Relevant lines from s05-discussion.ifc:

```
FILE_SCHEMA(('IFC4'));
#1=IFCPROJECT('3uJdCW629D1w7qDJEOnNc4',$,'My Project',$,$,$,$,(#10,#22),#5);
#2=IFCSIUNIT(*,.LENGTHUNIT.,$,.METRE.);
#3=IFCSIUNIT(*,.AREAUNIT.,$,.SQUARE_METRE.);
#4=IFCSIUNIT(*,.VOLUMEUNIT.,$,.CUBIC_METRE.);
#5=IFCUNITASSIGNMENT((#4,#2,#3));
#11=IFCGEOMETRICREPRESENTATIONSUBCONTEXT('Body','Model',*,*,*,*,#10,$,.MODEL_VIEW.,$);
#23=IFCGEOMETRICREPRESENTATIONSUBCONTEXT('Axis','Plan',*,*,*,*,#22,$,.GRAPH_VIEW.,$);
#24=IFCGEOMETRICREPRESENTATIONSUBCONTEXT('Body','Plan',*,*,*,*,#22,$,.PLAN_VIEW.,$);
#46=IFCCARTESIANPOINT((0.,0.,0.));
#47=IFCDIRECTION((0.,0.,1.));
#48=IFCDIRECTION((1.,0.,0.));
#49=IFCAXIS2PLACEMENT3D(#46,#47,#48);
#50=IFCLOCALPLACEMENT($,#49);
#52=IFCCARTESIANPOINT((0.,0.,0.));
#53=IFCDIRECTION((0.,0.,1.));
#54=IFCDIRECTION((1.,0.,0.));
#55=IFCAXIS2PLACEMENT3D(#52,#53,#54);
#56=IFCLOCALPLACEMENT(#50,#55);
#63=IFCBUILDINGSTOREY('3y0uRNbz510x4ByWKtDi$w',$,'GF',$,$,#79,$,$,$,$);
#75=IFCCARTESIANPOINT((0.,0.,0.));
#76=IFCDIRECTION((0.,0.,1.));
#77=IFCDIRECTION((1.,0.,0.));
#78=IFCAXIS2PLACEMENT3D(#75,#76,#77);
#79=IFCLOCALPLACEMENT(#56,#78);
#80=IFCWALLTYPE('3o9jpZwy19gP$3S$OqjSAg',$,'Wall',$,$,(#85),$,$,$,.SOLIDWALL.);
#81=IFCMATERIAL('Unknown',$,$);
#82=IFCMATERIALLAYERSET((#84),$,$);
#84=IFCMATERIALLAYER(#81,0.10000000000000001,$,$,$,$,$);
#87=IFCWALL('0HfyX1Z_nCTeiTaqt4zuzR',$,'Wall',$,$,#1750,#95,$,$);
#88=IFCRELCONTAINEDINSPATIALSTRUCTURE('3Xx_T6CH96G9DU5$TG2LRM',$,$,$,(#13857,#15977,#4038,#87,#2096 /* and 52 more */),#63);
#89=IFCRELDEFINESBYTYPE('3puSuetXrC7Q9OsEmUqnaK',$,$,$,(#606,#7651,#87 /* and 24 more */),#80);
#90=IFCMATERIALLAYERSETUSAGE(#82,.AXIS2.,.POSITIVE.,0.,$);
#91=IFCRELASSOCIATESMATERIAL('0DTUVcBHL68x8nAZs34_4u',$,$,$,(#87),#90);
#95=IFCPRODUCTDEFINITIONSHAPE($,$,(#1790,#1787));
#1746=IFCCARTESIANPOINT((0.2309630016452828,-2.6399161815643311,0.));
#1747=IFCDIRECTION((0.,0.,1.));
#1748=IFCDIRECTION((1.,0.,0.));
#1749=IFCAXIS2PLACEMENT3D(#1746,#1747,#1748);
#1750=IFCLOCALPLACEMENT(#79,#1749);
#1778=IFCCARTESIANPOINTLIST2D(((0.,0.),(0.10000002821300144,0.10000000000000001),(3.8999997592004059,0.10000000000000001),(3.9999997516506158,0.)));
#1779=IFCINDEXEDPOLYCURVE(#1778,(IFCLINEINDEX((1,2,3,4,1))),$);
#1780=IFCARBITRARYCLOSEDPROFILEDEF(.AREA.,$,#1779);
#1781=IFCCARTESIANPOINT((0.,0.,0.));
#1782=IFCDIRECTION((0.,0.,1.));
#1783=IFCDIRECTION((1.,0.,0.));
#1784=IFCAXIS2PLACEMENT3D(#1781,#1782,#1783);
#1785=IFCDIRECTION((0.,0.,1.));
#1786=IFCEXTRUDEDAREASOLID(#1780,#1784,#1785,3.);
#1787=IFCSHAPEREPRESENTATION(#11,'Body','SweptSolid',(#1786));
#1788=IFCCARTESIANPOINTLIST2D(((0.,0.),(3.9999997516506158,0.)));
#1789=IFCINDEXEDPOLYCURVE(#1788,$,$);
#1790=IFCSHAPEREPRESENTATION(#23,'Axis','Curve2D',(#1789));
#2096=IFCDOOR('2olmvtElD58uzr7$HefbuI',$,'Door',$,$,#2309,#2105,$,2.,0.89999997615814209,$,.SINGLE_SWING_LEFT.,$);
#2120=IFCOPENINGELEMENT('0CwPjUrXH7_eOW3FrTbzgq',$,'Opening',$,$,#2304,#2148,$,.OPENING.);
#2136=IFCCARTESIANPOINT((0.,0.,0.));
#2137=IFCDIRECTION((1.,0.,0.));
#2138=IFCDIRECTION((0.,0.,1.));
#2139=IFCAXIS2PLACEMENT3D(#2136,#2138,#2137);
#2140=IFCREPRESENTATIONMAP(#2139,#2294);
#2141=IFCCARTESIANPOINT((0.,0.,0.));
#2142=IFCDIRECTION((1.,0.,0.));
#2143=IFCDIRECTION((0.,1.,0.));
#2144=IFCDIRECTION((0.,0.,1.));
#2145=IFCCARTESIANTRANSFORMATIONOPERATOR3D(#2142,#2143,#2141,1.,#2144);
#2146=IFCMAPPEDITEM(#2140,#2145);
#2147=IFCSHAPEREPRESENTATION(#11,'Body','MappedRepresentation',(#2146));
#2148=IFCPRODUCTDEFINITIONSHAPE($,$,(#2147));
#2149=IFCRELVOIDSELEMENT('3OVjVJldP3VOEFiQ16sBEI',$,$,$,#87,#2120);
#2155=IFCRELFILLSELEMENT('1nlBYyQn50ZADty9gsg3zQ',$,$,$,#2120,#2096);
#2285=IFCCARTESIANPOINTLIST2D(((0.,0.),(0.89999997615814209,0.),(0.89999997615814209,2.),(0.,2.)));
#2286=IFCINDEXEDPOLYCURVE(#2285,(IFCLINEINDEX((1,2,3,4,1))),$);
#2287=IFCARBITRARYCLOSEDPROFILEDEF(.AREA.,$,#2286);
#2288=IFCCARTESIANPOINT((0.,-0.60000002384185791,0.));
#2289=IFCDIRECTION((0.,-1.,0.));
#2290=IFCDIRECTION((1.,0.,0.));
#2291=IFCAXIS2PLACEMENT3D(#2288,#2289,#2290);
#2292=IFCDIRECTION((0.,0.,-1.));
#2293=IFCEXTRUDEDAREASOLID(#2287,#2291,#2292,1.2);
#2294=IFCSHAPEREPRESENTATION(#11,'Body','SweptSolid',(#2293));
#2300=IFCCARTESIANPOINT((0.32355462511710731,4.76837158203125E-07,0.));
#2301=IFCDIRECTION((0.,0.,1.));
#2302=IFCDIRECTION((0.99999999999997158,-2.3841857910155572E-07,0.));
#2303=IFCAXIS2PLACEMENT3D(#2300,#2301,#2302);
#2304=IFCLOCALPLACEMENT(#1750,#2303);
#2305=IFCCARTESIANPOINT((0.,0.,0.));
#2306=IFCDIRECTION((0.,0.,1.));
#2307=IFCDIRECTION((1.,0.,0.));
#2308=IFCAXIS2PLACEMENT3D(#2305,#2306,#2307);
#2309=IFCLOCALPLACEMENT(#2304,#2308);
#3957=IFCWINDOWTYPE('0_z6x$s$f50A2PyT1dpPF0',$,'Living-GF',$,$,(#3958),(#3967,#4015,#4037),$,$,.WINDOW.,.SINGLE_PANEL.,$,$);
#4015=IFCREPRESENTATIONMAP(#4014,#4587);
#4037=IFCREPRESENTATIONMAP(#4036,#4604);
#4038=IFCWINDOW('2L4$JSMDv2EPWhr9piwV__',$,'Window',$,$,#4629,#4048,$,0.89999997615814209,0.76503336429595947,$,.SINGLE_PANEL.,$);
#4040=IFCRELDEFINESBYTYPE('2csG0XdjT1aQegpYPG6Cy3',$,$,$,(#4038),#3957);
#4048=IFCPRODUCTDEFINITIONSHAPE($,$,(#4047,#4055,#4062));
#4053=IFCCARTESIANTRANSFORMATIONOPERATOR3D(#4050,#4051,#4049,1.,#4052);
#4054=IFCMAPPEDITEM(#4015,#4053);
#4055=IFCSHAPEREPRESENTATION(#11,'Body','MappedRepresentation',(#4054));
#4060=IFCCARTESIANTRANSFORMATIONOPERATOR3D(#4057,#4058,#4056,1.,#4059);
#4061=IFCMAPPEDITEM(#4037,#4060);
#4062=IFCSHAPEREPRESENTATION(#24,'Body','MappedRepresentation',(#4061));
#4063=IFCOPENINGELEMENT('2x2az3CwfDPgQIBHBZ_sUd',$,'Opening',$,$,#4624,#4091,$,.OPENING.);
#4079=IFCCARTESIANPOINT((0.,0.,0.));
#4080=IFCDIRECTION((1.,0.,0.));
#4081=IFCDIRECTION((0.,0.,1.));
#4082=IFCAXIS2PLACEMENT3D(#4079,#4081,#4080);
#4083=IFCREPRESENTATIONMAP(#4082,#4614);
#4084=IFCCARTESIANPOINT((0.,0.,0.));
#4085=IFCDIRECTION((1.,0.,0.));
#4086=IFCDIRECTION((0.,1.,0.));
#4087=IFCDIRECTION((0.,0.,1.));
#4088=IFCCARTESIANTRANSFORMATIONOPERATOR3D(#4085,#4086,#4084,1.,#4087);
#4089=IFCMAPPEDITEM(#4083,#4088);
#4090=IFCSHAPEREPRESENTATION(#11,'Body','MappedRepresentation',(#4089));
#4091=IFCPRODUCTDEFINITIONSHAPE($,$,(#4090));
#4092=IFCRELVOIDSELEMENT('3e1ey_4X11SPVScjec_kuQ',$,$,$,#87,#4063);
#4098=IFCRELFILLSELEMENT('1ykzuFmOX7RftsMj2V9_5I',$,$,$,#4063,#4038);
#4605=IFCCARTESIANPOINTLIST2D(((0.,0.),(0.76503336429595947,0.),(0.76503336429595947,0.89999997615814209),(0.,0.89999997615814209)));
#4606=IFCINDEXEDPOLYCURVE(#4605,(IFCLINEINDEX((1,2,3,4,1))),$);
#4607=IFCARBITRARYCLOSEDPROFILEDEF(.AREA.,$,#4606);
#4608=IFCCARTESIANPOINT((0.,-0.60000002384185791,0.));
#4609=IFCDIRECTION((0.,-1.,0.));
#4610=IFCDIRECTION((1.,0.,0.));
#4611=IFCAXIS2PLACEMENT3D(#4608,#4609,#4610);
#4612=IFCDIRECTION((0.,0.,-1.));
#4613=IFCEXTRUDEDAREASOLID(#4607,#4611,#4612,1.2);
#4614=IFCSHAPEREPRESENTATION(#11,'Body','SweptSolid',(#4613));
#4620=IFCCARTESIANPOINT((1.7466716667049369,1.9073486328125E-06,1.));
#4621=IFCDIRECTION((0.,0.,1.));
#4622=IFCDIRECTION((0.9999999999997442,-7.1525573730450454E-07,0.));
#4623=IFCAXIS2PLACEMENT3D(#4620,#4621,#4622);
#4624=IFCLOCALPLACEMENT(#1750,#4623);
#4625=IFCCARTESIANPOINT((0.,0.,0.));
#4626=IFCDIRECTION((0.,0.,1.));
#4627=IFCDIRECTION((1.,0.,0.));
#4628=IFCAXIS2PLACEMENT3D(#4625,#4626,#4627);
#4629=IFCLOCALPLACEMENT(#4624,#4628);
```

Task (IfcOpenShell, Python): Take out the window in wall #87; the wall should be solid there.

```python
import ifcopenshell
import ifcopenshell.api.feature
import ifcopenshell.api.root
import ifcopenshell.geom
import ifcopenshell.util.shape

model = ifcopenshell.open("s05-discussion.ifc")
settings = ifcopenshell.geom.settings()


def volume(element):
    """Net volume in cubic metres, openings subtracted."""
    shape = ifcopenshell.geom.create_shape(settings, element)
    return ifcopenshell.util.shape.get_volume(shape.geometry)


window = model.by_guid("2L4$JSMDv2EPWhr9piwV__")
opening = window.FillsVoids[0].RelatingOpeningElement
wall = opening.VoidsElements[0].RelatingBuildingElement
before = volume(wall)

ifcopenshell.api.root.remove_product(model, product=window)
ifcopenshell.api.feature.remove_feature(model, feature=opening)

after = volume(wall)

print(f"wall volume {before:.3f} -> {after:.3f} m3")

model.write("s05-discussion_rev.ifc")
```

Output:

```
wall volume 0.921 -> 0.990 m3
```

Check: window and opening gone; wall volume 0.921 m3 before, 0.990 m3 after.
